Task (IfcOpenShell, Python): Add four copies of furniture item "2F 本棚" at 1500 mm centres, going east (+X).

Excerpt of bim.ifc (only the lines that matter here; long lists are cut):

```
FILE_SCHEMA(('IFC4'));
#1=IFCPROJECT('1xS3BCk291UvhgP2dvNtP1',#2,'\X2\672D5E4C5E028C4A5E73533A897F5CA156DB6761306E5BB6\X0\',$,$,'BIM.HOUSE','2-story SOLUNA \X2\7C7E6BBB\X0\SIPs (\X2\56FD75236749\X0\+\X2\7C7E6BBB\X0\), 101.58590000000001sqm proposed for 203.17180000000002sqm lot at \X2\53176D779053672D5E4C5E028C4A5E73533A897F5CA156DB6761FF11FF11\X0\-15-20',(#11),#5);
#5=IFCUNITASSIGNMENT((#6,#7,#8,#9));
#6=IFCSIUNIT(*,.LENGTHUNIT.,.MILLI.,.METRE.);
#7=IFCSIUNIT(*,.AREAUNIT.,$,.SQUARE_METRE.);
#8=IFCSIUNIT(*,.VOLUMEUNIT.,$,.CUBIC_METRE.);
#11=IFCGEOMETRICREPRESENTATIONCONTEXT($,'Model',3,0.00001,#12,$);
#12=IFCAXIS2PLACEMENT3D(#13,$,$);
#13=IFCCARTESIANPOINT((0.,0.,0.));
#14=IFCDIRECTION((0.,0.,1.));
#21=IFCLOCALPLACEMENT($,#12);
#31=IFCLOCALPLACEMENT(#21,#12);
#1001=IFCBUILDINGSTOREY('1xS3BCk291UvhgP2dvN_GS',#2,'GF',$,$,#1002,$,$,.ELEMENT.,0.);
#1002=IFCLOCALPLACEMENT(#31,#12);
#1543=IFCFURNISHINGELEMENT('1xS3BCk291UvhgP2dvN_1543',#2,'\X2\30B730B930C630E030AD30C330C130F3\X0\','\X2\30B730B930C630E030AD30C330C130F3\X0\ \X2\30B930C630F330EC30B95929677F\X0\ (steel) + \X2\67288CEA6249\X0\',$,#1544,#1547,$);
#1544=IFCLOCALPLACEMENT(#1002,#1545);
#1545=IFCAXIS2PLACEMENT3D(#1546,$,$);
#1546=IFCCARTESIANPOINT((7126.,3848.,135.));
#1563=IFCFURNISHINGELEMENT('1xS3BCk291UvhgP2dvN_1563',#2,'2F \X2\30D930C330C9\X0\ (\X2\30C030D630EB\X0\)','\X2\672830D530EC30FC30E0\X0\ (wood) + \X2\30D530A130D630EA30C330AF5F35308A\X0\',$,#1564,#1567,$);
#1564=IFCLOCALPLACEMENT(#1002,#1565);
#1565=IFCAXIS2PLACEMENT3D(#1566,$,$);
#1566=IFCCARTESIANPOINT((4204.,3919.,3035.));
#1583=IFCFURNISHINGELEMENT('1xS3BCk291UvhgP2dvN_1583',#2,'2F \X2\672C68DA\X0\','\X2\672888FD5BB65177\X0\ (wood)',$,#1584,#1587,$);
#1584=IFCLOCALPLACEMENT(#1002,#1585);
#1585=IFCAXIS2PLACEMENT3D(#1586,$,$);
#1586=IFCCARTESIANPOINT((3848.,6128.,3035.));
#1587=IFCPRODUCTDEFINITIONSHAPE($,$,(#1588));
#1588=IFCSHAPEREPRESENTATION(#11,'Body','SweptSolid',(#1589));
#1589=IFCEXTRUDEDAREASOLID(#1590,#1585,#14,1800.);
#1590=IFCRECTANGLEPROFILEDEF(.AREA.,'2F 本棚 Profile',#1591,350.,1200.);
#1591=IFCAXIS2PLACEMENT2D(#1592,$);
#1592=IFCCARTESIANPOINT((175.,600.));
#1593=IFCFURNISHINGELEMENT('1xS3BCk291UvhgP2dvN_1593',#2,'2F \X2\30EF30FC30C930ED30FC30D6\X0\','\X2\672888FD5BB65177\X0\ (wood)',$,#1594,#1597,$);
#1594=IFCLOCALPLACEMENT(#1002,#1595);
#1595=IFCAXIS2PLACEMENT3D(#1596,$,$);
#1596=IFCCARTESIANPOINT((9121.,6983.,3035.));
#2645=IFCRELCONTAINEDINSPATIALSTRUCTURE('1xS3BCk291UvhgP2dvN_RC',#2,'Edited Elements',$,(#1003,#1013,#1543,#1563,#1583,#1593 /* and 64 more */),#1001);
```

```python
import numpy as np
import ifcopenshell
import ifcopenshell.api.geometry
import ifcopenshell.api.root
import ifcopenshell.util.element
import ifcopenshell.util.placement

model = ifcopenshell.open("bim.ifc")


def reuse_history(source, copy):
    """copy_class also copies each property set's owner history, people and application; keep the originals."""
    for rel in copy.IsDefinedBy:
        if rel.is_a("IfcRelDefinesByProperties") and (history := rel.RelatingPropertyDefinition.OwnerHistory):
            rel.RelatingPropertyDefinition.OwnerHistory = source.OwnerHistory
            ifcopenshell.util.element.remove_deep2(model, history)


source = model.by_guid("1xS3BCk291UvhgP2dvN_1583")
base = ifcopenshell.util.placement.get_local_placement(source.ObjectPlacement)
step = np.array([1.0, 0.0, 0.0]) * 1500.0

for i in range(1, 5):
    copy = ifcopenshell.api.root.copy_class(model, product=source)
    copy.Representation = ifcopenshell.util.element.copy_deep(
        model, source.Representation, exclude=["IfcGeometricRepresentationContext", "IfcRepresentationMap"]
    )
    reuse_history(source, copy)
    matrix = base.copy()
    matrix[:3, 3] += i * step
    print("added at", matrix[:3, 3].round(3) + 0.0)
    ifcopenshell.api.geometry.edit_object_placement(model, product=copy, matrix=matrix, is_si=False)

model.write("bim-out.ifc")
```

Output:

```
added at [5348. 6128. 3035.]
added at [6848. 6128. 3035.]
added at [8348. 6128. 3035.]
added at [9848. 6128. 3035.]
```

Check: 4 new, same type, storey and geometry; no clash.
